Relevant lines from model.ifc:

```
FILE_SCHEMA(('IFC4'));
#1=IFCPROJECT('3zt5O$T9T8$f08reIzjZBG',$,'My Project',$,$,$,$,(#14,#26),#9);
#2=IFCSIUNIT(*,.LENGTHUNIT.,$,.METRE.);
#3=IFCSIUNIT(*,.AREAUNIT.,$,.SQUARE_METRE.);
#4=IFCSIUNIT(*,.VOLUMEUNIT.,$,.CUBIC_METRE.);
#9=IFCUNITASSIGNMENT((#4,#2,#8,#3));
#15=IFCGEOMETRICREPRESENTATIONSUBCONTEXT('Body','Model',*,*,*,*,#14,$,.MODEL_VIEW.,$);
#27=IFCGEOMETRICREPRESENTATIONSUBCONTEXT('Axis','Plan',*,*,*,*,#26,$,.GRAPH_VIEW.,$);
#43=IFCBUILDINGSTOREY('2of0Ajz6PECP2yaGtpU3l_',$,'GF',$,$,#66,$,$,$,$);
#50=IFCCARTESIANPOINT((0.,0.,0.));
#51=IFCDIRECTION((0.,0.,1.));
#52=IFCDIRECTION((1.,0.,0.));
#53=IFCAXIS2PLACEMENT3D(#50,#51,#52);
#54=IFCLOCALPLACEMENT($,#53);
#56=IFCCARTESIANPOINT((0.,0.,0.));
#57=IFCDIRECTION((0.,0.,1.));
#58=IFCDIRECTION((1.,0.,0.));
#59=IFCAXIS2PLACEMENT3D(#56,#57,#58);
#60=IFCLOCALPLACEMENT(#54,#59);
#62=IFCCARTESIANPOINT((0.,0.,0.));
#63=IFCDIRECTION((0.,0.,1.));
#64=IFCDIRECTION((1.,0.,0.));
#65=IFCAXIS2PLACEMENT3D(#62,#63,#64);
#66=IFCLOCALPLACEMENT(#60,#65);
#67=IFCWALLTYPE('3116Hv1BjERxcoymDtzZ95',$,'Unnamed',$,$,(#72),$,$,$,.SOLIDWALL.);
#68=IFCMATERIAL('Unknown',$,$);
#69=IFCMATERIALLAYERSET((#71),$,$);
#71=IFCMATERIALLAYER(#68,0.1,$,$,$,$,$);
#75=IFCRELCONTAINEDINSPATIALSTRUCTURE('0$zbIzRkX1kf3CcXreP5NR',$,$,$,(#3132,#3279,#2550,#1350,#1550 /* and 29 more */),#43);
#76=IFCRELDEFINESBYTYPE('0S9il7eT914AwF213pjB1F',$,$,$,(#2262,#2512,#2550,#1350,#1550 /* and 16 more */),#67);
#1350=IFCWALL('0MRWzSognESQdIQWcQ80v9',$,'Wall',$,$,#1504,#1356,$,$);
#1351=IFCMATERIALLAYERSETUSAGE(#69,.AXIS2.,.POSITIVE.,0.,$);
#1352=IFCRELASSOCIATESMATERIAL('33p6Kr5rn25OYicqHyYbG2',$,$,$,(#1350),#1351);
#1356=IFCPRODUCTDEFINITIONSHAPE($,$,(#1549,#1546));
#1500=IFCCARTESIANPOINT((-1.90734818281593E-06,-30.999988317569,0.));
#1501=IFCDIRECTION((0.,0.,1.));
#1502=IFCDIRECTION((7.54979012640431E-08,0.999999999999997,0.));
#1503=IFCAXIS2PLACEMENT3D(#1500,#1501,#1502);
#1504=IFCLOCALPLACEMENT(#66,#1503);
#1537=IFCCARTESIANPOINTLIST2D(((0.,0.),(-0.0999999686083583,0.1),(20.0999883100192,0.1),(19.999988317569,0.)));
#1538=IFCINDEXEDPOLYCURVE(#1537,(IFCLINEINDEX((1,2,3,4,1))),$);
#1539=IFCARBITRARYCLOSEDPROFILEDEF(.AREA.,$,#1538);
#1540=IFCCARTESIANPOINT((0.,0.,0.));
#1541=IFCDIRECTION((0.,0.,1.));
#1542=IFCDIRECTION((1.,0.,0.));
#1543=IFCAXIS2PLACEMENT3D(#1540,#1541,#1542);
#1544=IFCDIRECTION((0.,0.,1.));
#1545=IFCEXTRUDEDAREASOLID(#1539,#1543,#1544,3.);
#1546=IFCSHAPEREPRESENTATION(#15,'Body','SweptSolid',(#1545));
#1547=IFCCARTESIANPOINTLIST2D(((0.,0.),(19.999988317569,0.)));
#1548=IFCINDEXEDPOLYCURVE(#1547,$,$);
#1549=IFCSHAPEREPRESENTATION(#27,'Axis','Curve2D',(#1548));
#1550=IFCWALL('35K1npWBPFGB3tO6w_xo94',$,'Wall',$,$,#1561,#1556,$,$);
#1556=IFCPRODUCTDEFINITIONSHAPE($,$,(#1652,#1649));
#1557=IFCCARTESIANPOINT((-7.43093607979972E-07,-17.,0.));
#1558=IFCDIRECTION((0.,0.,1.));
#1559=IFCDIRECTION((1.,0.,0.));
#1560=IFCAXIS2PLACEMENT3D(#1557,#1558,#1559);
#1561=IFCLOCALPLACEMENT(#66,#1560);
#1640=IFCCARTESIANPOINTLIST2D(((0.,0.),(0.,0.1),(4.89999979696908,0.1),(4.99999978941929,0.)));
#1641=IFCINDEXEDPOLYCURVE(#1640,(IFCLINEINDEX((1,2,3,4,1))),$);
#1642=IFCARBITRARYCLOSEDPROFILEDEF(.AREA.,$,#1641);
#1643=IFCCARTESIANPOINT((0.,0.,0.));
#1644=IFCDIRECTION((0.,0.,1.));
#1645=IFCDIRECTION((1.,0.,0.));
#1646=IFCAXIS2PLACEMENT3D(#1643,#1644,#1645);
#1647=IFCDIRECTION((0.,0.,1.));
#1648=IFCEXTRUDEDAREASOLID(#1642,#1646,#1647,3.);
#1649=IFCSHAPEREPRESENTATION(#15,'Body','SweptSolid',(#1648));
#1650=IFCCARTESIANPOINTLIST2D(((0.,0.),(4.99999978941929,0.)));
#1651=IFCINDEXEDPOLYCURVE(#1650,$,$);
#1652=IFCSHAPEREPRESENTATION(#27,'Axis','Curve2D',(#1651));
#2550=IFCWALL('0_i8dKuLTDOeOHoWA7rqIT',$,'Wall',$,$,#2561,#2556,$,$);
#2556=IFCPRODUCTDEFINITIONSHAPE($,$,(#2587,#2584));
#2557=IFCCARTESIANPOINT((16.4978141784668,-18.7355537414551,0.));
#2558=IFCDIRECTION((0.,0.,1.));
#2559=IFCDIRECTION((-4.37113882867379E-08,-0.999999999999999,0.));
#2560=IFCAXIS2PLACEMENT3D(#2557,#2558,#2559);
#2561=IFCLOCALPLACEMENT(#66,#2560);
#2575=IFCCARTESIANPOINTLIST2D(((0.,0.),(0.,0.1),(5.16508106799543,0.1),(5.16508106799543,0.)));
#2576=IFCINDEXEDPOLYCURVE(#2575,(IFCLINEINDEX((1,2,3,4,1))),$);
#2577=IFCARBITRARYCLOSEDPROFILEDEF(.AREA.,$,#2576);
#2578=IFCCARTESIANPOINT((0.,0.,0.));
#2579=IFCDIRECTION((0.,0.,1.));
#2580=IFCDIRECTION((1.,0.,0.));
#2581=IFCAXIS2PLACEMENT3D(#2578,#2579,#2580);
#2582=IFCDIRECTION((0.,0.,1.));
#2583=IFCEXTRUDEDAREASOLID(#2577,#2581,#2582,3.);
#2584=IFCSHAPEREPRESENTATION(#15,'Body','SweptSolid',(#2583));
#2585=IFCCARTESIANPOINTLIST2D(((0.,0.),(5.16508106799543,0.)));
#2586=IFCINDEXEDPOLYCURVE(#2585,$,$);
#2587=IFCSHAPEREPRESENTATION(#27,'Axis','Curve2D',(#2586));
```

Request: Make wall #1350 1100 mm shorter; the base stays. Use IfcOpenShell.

```python
import ifcopenshell
import ifcopenshell.geom
import ifcopenshell.util.representation
import ifcopenshell.util.shape

model = ifcopenshell.open("model.ifc")
settings = ifcopenshell.geom.settings()


def volume(element):
    """Net volume in cubic metres, openings subtracted."""
    shape = ifcopenshell.geom.create_shape(settings, element)
    return ifcopenshell.util.shape.get_volume(shape.geometry)


wall = model.by_guid("0MRWzSognESQdIQWcQ80v9")
before = volume(wall)

body = ifcopenshell.util.representation.get_representation(wall, "Model", "Body")
solid = body.Items[0]
old_height = solid.Depth
solid.Depth -= 1.1
after = volume(wall)

print(f"height {old_height:g} -> {solid.Depth:g}, volume {before:.3f} -> {after:.3f} m3")

model.write("model_updated.ifc")
```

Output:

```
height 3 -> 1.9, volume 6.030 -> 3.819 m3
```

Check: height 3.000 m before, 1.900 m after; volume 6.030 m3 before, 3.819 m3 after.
